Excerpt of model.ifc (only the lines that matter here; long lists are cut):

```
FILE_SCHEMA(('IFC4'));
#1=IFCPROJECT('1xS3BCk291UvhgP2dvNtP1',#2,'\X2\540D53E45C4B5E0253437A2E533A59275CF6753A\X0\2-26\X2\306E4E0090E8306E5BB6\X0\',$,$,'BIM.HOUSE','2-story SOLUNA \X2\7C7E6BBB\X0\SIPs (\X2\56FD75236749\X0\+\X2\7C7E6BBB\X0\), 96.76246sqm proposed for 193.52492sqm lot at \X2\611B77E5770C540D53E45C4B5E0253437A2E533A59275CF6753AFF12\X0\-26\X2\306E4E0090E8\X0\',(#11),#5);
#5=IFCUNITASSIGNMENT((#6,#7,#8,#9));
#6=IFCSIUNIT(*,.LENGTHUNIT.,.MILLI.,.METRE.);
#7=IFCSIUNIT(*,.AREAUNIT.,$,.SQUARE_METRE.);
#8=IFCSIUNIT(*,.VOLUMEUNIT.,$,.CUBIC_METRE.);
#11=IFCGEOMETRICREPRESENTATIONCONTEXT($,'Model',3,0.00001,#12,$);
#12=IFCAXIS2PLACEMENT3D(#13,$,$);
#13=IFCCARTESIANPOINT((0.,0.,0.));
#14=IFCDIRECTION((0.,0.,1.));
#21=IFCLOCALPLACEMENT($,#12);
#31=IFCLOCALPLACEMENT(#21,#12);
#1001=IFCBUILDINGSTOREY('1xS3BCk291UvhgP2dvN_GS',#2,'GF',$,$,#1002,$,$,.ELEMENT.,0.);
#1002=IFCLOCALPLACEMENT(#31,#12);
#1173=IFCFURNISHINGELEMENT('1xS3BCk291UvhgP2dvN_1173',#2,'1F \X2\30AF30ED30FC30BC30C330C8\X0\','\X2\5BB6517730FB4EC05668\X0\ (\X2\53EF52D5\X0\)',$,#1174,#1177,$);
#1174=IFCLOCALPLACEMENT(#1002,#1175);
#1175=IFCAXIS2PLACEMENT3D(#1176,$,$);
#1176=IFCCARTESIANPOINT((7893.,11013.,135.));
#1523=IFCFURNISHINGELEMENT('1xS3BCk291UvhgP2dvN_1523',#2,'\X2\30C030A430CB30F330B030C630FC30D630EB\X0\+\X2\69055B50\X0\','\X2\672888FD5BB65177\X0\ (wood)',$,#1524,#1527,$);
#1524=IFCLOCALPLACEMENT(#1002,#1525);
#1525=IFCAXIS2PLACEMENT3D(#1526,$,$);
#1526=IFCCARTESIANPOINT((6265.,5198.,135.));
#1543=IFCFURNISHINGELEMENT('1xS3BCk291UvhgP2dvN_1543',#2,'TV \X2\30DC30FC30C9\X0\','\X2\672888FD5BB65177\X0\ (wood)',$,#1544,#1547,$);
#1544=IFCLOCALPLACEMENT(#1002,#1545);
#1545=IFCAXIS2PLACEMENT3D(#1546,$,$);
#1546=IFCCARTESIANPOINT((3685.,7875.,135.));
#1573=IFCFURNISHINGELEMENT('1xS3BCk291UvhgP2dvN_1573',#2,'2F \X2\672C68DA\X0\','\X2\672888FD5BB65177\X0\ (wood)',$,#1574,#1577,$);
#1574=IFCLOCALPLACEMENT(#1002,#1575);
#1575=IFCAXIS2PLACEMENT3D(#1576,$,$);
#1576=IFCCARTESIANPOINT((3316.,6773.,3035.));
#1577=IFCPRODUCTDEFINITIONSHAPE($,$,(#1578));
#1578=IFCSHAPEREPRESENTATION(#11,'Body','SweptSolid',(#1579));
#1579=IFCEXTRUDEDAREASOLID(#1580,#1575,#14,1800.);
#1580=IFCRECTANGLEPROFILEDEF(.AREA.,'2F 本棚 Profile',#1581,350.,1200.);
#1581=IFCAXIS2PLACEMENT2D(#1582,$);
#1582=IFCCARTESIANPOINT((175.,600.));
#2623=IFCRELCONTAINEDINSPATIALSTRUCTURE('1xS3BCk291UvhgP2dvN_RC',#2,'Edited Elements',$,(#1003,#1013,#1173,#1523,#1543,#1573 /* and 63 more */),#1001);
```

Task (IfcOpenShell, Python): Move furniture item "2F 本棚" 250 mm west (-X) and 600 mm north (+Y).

```python
import ifcopenshell
import ifcopenshell.api.geometry
import ifcopenshell.util.placement
import ifcopenshell.util.unit

model = ifcopenshell.open("model.ifc")
unit_scale = ifcopenshell.util.unit.calculate_unit_scale(model)

item = model.by_id(1573)
matrix = ifcopenshell.util.placement.get_local_placement(item.ObjectPlacement)
matrix[0, 3] -= 0.25 / unit_scale
matrix[1, 3] += 0.6 / unit_scale
ifcopenshell.api.geometry.edit_object_placement(model, product=item, matrix=matrix, is_si=False)

print(ifcopenshell.util.placement.get_local_placement(item.ObjectPlacement).round(3) + 0.0)

model.write("model_updated.ifc")
```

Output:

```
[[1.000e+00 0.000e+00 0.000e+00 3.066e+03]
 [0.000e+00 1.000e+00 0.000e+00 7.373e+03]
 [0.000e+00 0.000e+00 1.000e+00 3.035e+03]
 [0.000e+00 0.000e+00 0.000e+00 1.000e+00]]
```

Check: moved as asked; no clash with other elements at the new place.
